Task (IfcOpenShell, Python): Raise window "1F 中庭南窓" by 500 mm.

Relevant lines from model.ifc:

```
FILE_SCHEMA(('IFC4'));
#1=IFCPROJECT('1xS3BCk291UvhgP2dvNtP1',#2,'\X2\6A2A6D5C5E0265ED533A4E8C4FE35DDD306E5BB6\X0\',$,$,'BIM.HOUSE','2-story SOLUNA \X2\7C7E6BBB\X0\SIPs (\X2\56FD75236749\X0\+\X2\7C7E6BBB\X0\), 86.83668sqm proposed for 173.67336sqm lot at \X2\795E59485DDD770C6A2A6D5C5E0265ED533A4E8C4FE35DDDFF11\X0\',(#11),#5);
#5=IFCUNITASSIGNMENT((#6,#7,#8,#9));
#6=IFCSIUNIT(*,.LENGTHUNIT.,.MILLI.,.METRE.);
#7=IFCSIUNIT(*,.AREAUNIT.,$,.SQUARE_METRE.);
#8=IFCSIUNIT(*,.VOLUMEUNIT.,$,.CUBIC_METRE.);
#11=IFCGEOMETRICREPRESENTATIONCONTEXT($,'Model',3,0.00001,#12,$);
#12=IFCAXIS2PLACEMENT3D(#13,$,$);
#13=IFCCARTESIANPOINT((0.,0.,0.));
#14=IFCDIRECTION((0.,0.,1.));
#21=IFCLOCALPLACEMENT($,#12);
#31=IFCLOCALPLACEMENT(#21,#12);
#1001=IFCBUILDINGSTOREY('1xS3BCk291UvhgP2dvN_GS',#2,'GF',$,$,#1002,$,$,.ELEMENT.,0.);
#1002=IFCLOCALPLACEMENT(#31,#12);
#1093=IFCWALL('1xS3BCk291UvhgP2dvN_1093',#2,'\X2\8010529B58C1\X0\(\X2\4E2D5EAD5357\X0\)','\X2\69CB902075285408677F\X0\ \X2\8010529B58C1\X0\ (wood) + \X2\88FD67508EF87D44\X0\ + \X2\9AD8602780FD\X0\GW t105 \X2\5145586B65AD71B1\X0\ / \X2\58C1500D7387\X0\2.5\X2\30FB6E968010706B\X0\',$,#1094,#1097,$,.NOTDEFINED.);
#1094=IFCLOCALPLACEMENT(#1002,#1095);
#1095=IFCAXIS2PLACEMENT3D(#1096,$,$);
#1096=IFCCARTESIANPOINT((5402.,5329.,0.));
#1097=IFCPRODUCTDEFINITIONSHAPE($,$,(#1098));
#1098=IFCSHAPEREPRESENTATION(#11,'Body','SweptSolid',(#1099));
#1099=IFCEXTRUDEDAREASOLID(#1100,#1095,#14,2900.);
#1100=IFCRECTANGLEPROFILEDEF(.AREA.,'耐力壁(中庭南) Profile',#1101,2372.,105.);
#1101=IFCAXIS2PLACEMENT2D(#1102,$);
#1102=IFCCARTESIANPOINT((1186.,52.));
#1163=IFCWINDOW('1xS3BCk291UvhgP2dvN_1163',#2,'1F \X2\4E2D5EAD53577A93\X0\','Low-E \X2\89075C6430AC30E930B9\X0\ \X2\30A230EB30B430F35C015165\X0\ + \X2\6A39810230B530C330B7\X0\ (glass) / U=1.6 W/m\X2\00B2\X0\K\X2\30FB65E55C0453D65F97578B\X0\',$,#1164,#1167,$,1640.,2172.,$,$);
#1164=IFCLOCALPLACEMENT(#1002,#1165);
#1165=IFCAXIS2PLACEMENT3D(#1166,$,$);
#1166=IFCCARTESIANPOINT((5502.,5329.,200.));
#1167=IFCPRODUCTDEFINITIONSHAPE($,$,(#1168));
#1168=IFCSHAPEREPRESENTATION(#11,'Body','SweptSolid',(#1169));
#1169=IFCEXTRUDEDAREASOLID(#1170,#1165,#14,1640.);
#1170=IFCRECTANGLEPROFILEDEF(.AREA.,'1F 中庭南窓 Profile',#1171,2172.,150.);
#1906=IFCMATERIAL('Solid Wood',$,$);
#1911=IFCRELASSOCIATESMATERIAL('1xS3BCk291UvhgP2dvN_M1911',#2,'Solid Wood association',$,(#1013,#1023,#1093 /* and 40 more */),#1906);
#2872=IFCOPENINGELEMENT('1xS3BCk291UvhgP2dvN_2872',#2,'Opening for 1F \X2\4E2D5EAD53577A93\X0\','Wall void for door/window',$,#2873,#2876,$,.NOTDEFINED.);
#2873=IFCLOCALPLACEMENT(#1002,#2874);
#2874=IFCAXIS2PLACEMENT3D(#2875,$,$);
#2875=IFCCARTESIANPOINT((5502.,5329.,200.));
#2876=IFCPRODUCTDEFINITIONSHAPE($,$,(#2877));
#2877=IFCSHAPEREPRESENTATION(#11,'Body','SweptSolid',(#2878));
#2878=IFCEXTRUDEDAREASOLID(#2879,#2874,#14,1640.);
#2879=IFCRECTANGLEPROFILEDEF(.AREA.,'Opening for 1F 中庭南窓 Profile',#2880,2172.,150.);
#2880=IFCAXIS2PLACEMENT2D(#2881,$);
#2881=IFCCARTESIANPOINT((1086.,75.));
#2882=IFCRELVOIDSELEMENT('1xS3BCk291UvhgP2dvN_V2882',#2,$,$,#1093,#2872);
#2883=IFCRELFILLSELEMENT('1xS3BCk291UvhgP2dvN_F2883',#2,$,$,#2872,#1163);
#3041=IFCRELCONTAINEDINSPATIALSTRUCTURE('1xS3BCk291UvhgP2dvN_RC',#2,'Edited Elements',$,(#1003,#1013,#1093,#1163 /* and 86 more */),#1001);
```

```python
import numpy as np
import ifcopenshell
import ifcopenshell.api.geometry
import ifcopenshell.util.placement
import ifcopenshell.util.unit

model = ifcopenshell.open("model.ifc")
unit_scale = ifcopenshell.util.unit.calculate_unit_scale(model)

window = model.by_guid("1xS3BCk291UvhgP2dvN_1163")
opening = window.FillsVoids[0].RelatingOpeningElement
dz = 500.0

shift = np.array([0.0, 0.0, dz])
# The window is not placed relative to its opening, so move both.
for product in (opening, window):
    matrix = ifcopenshell.util.placement.get_local_placement(product.ObjectPlacement)
    matrix[:3, 3] += shift
    ifcopenshell.api.geometry.edit_object_placement(model, product=product, matrix=matrix, is_si=False)

print(f"moved by {dz * unit_scale:+.3f} m")

model.write("model_v2.ifc")
```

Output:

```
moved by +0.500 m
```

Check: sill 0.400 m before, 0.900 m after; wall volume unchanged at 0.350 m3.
